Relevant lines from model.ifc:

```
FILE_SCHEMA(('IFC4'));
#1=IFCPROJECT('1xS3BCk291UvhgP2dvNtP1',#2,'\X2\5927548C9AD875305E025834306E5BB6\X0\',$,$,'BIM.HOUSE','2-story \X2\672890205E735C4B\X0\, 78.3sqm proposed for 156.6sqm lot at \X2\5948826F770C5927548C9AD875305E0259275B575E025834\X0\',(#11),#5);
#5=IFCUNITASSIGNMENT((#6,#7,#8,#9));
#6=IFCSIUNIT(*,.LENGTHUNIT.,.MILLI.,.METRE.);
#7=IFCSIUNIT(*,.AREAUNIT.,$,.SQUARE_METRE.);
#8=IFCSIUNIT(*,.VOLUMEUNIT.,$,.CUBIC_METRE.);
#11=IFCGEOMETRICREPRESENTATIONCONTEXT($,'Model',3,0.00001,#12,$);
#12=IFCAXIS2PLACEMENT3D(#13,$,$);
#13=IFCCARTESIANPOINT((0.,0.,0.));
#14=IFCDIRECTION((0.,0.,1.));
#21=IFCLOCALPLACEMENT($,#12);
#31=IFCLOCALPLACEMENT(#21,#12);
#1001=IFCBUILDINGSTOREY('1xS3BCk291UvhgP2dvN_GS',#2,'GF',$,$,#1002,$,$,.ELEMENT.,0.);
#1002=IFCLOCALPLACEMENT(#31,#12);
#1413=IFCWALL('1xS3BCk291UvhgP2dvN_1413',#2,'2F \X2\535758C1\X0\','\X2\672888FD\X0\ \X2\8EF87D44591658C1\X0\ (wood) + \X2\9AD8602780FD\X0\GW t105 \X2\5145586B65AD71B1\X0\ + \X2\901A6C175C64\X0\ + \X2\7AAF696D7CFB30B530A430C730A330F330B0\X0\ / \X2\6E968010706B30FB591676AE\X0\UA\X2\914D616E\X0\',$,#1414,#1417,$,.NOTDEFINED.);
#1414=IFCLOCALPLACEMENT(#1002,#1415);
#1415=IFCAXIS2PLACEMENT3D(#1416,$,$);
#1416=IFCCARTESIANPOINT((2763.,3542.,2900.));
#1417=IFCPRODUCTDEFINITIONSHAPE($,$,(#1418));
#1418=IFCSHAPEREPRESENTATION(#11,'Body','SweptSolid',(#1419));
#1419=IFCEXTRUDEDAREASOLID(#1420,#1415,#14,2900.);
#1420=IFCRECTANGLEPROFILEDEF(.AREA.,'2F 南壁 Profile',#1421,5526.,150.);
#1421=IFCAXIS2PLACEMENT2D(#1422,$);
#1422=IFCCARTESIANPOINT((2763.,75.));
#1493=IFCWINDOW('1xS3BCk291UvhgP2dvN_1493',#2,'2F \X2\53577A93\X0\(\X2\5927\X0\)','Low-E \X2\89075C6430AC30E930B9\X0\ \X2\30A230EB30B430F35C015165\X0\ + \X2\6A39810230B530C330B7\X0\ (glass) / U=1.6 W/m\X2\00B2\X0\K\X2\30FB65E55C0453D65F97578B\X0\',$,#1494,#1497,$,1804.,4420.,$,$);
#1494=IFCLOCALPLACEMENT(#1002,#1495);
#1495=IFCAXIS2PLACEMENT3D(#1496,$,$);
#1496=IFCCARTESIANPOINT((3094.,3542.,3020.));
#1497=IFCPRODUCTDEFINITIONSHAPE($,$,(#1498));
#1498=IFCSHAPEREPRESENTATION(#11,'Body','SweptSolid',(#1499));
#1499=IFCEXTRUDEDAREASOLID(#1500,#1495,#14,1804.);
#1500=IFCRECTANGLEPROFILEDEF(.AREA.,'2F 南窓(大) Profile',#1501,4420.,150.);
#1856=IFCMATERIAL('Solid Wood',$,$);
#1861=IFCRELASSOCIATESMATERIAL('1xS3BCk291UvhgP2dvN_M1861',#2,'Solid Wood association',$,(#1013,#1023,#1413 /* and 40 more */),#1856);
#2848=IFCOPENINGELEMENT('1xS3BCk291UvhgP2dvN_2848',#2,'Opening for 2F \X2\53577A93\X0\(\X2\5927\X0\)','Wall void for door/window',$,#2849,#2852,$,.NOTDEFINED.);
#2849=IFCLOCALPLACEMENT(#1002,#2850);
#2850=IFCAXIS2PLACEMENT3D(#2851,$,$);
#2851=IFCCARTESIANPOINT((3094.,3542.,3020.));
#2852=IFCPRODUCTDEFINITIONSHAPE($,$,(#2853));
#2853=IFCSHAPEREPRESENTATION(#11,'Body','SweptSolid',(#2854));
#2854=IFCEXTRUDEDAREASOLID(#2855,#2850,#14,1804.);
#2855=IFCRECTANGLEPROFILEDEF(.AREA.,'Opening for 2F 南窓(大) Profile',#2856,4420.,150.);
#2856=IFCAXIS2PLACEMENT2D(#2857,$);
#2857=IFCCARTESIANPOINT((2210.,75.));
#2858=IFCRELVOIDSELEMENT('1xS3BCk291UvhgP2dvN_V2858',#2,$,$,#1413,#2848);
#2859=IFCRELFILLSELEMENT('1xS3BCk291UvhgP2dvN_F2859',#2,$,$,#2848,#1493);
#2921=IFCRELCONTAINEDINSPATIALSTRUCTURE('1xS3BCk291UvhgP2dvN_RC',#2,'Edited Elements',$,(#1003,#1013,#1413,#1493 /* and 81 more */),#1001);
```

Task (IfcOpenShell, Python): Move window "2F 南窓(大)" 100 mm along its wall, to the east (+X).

```python
import ifcopenshell
import ifcopenshell.api.geometry
import ifcopenshell.util.placement
import ifcopenshell.util.unit

model = ifcopenshell.open("model.ifc")
unit_scale = ifcopenshell.util.unit.calculate_unit_scale(model)

window = model.by_guid("1xS3BCk291UvhgP2dvN_1493")
opening = window.FillsVoids[0].RelatingOpeningElement
wall = opening.VoidsElements[0].RelatingBuildingElement

wall_matrix = ifcopenshell.util.placement.get_local_placement(wall.ObjectPlacement)
shift = wall_matrix[:3, 0] * 0.1 / unit_scale
before = ifcopenshell.util.placement.get_local_placement(window.ObjectPlacement)[:3, 3].copy()

# The window is not placed relative to its opening, so move both.
for product in (opening, window):
    matrix = ifcopenshell.util.placement.get_local_placement(product.ObjectPlacement)
    matrix[:3, 3] += shift
    ifcopenshell.api.geometry.edit_object_placement(model, product=product, matrix=matrix, is_si=False)

after = ifcopenshell.util.placement.get_local_placement(window.ObjectPlacement)[:3, 3]
print("window moved by", (after - before).round(3) + 0.0)

model.write("model_updated.ifc")
```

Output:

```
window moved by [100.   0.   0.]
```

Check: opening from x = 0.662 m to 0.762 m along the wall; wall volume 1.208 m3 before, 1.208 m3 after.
